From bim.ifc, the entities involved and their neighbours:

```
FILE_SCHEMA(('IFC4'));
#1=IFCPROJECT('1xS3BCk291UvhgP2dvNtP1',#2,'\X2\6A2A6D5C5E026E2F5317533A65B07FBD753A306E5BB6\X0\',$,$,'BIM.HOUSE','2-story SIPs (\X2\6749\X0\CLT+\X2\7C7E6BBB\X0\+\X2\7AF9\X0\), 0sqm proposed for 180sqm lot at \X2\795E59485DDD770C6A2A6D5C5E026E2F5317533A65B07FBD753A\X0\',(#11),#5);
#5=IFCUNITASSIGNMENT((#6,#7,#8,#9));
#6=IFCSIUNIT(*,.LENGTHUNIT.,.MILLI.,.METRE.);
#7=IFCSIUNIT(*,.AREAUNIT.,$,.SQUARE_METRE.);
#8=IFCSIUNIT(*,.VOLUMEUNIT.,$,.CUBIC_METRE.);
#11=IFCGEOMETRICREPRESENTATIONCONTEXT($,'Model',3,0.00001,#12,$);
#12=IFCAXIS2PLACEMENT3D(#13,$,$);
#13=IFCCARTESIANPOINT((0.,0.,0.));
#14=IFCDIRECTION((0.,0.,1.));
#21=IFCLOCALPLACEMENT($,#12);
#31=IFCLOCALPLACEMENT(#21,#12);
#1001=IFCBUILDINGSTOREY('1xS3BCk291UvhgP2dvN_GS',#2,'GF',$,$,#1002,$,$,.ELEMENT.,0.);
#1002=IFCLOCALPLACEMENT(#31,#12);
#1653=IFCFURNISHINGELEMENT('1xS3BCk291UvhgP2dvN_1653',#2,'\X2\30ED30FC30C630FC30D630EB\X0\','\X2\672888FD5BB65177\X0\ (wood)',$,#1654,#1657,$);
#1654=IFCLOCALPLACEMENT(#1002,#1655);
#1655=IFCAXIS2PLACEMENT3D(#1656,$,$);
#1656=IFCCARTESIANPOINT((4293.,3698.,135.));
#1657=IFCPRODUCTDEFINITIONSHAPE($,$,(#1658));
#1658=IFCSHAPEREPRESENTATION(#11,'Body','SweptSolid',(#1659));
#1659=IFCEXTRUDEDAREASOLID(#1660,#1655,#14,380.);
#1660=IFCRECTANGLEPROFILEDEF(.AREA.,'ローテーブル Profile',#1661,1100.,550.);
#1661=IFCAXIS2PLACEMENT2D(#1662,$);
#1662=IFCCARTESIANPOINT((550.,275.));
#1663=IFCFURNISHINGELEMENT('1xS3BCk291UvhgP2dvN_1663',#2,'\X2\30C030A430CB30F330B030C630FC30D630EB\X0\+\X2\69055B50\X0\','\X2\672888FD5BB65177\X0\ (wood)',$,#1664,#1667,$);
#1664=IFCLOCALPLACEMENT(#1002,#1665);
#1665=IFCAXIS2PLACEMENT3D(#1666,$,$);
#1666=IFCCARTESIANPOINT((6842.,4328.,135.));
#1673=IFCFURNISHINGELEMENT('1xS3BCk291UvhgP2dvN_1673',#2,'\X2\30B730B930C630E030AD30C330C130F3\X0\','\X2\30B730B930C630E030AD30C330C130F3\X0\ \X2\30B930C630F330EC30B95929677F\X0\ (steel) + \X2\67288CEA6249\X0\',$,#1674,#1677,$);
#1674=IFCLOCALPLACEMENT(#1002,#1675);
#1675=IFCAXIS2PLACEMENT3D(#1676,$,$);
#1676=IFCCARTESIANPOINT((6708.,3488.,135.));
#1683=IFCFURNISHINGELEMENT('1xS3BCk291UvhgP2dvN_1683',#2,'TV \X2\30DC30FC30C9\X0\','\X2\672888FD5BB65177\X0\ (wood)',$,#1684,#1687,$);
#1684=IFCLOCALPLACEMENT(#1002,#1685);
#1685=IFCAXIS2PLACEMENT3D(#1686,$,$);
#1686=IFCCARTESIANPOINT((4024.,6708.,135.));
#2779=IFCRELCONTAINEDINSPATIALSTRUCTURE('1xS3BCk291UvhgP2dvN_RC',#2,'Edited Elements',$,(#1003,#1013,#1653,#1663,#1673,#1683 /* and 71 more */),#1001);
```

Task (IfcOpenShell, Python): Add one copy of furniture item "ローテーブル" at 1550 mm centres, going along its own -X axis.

```python
import ifcopenshell
import ifcopenshell.api.geometry
import ifcopenshell.api.root
import ifcopenshell.util.element
import ifcopenshell.util.placement

model = ifcopenshell.open("bim.ifc")


def reuse_history(source, copy):
    """copy_class also copies each property set's owner history, people and application; keep the originals."""
    for rel in copy.IsDefinedBy:
        if rel.is_a("IfcRelDefinesByProperties") and (history := rel.RelatingPropertyDefinition.OwnerHistory):
            rel.RelatingPropertyDefinition.OwnerHistory = source.OwnerHistory
            ifcopenshell.util.element.remove_deep2(model, history)


source = model.by_id(1653)
base = ifcopenshell.util.placement.get_local_placement(source.ObjectPlacement)
step = -base[:3, 0] * 1550.0

for i in range(1, 2):
    copy = ifcopenshell.api.root.copy_class(model, product=source)
    copy.Representation = ifcopenshell.util.element.copy_deep(
        model, source.Representation, exclude=["IfcGeometricRepresentationContext", "IfcRepresentationMap"]
    )
    reuse_history(source, copy)
    matrix = base.copy()
    matrix[:3, 3] += i * step
    print("added at", matrix[:3, 3].round(3) + 0.0)
    ifcopenshell.api.geometry.edit_object_placement(model, product=copy, matrix=matrix, is_si=False)

model.write("bim-out.ifc")
```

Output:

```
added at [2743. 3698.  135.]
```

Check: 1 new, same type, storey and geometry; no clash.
